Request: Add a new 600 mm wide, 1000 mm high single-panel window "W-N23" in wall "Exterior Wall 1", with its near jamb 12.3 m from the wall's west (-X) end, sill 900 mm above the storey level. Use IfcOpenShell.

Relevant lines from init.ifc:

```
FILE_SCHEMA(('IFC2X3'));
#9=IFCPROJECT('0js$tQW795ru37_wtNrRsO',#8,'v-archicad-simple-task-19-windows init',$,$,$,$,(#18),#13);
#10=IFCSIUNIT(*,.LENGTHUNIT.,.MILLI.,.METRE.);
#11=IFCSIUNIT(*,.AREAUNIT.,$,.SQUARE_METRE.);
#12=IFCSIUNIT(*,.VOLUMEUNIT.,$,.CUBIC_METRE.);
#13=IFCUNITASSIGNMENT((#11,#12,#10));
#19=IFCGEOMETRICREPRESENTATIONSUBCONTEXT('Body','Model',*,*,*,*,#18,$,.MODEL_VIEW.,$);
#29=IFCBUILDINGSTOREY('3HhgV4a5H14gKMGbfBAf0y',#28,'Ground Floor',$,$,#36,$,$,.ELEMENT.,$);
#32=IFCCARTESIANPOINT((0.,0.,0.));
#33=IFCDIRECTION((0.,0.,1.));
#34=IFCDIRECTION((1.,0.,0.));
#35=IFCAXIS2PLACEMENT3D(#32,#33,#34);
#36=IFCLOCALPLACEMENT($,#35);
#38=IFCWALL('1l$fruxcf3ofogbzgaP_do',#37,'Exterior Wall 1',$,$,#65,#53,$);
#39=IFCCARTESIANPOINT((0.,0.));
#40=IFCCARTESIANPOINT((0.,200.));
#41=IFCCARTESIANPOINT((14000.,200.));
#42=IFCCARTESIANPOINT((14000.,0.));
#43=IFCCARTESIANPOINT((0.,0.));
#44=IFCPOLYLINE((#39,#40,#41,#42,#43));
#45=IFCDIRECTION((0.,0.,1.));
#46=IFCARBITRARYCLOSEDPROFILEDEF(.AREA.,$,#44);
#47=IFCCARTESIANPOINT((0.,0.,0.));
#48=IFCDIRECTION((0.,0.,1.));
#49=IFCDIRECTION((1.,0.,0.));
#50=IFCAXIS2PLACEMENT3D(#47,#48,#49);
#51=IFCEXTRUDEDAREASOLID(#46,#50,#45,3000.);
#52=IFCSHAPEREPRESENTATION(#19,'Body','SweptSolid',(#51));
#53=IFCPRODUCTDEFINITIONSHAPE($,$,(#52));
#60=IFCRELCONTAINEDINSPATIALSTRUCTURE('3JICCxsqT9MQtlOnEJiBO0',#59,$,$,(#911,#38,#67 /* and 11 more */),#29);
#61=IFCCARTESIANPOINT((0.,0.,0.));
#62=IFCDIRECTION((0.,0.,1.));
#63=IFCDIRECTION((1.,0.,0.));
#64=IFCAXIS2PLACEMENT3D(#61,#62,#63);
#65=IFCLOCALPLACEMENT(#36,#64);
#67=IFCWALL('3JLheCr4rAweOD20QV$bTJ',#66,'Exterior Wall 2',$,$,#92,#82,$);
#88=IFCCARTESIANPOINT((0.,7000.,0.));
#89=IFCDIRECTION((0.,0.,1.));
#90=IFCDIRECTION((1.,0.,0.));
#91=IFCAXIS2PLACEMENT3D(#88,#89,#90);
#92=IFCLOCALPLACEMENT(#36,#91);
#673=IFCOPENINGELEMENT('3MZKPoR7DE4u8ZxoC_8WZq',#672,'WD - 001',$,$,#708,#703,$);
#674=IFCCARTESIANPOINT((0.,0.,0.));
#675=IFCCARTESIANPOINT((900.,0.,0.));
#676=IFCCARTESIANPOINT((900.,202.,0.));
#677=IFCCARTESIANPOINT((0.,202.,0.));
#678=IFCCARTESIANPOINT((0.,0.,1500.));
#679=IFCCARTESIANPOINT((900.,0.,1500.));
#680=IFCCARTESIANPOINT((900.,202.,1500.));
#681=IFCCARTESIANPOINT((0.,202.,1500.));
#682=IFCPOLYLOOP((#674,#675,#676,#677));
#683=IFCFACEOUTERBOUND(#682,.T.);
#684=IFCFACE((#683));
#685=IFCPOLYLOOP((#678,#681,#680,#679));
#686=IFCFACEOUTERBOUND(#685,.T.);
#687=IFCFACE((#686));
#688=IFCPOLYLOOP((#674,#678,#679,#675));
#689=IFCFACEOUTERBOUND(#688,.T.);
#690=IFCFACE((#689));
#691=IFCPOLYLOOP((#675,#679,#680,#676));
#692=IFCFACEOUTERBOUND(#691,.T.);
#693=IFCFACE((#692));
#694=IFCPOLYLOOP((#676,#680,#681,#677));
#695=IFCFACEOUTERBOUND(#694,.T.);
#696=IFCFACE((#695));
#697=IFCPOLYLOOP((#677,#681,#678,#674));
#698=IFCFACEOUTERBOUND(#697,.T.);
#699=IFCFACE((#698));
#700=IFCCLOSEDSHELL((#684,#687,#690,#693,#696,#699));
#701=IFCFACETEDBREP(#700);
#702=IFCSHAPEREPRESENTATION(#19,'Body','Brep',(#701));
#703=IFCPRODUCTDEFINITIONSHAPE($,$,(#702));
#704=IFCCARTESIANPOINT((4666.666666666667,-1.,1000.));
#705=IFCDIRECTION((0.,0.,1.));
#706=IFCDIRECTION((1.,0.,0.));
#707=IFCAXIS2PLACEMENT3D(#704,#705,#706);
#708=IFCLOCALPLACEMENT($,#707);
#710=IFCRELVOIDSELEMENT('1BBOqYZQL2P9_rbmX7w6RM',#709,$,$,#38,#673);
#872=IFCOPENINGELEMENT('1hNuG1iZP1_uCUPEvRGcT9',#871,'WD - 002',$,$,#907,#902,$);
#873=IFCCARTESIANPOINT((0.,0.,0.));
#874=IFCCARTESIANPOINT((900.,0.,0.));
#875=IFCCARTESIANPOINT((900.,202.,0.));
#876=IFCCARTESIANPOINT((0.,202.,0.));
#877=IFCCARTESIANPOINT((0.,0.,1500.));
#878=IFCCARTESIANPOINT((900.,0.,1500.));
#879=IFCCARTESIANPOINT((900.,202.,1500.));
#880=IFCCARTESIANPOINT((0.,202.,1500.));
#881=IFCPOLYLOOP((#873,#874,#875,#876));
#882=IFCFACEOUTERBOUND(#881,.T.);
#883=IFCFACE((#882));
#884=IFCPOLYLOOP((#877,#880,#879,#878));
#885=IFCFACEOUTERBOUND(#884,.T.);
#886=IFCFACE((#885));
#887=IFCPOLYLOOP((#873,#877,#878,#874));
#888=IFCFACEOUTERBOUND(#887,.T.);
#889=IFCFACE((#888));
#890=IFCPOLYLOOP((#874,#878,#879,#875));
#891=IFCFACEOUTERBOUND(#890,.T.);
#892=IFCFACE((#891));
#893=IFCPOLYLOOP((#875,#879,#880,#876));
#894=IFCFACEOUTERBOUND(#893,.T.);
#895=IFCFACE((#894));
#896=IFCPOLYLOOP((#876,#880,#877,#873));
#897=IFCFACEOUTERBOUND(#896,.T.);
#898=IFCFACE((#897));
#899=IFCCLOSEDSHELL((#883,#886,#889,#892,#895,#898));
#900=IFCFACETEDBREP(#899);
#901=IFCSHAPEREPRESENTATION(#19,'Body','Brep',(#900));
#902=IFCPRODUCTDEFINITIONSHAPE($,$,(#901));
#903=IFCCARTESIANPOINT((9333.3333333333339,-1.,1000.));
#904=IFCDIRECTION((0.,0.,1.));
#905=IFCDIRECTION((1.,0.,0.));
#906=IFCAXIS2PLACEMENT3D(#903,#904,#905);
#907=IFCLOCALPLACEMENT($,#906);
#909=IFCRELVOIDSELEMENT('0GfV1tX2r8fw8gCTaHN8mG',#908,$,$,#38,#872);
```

```python
import numpy as np
import ifcopenshell
import ifcopenshell.api.feature
import ifcopenshell.api.geometry
import ifcopenshell.api.root
import ifcopenshell.api.spatial
import ifcopenshell.api.type
import ifcopenshell.geom
import ifcopenshell.util.element
import ifcopenshell.util.placement
import ifcopenshell.util.representation
import ifcopenshell.util.shape
import ifcopenshell.util.unit

model = ifcopenshell.open("init.ifc")
unit_scale = ifcopenshell.util.unit.calculate_unit_scale(model)
settings = ifcopenshell.geom.settings()


def volume(element):
    """Net volume in cubic metres, openings subtracted."""
    shape = ifcopenshell.geom.create_shape(settings, element)
    return ifcopenshell.util.shape.get_volume(shape.geometry)


wall = model.by_guid("1l$fruxcf3ofogbzgaP_do")
storey = ifcopenshell.util.element.get_container(wall, ifc_class="IfcBuildingStorey")
context = ifcopenshell.util.representation.get_context(model, "Model", "Body", "MODEL_VIEW")
before = volume(wall)

width, height, from_end, sill = 0.6, 1, 12.3, 0.9  # metres

# The wall runs along its own X axis, and the end named is its -X end.
wall_shape = ifcopenshell.geom.create_shape(settings, wall)
x, y, z = ifcopenshell.util.shape.get_vertices(wall_shape.geometry).T
start = x.min() + from_end
face, thickness = float(y.min()), float(y.max() - y.min())
wall_matrix = ifcopenshell.util.placement.get_local_placement(wall.ObjectPlacement)
level = ifcopenshell.util.placement.get_local_placement(storey.ObjectPlacement)[2, 3]


def in_wall(x, y):
    """Placement at x, y metres in the wall's axes, at sill height."""
    matrix = wall_matrix.copy()
    matrix[:, 3] = wall_matrix @ np.array([x / unit_scale, y / unit_scale, 0.0, 1.0])
    matrix[2, 3] = level + sill / unit_scale
    return matrix


# Opening: a box that overshoots both wall faces by 50 mm.
opening = ifcopenshell.api.root.create_entity(model, ifc_class="IfcOpeningElement")
box = ifcopenshell.api.geometry.add_wall_representation(
    model, context=context, length=width, height=height, thickness=thickness + 0.1
)
ifcopenshell.api.geometry.assign_representation(model, product=opening, representation=box)
ifcopenshell.api.geometry.edit_object_placement(model, product=opening, matrix=in_wall(start, face - 0.05), is_si=False)
ifcopenshell.api.feature.add_feature(model, feature=opening, element=wall)

window = ifcopenshell.api.root.create_entity(model, ifc_class="IfcWindow", name="W-N23")
window.OverallWidth, window.OverallHeight = width / unit_scale, height / unit_scale
body = ifcopenshell.api.geometry.add_window_representation(
    model,
    context=context,
    overall_width=window.OverallWidth,
    overall_height=window.OverallHeight,
    partition_type="SINGLE_PANEL",
)
ifcopenshell.api.geometry.assign_representation(model, product=window, representation=body)
ifcopenshell.api.spatial.assign_container(model, products=[window], relating_structure=storey)
fills = ifcopenshell.api.feature.add_filling(model, opening=opening, element=window)
fills.OwnerHistory = window.OwnerHistory  # required in IFC2X3

# IFC2X3 keeps the operation on the window style.
style = ifcopenshell.api.root.create_entity(model, ifc_class="IfcWindowStyle", name="W-N23")
style.OperationType, style.ConstructionType = "SINGLE_PANEL", "NOTDEFINED"
style.ParameterTakesPrecedence = style.Sizeable = False
ifcopenshell.api.type.assign_type(model, related_objects=[window], relating_type=style)

# Centre the window in the wall's thickness.
ifcopenshell.api.geometry.edit_object_placement(model, product=window, matrix=in_wall(start, face), is_si=False)
window_shape = ifcopenshell.geom.create_shape(settings, window)
depth = ifcopenshell.util.shape.get_vertices(window_shape.geometry)[:, 1]
offset = face + thickness / 2 - (depth.min() + depth.max()) / 2
ifcopenshell.api.geometry.edit_object_placement(model, product=window, matrix=in_wall(start, offset), is_si=False)

after = volume(wall)

print(f"wall volume {before:.3f} -> {after:.3f} m3")

model.write("init_rev.ifc")
```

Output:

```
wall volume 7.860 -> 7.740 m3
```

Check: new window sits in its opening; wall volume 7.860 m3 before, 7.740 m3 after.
